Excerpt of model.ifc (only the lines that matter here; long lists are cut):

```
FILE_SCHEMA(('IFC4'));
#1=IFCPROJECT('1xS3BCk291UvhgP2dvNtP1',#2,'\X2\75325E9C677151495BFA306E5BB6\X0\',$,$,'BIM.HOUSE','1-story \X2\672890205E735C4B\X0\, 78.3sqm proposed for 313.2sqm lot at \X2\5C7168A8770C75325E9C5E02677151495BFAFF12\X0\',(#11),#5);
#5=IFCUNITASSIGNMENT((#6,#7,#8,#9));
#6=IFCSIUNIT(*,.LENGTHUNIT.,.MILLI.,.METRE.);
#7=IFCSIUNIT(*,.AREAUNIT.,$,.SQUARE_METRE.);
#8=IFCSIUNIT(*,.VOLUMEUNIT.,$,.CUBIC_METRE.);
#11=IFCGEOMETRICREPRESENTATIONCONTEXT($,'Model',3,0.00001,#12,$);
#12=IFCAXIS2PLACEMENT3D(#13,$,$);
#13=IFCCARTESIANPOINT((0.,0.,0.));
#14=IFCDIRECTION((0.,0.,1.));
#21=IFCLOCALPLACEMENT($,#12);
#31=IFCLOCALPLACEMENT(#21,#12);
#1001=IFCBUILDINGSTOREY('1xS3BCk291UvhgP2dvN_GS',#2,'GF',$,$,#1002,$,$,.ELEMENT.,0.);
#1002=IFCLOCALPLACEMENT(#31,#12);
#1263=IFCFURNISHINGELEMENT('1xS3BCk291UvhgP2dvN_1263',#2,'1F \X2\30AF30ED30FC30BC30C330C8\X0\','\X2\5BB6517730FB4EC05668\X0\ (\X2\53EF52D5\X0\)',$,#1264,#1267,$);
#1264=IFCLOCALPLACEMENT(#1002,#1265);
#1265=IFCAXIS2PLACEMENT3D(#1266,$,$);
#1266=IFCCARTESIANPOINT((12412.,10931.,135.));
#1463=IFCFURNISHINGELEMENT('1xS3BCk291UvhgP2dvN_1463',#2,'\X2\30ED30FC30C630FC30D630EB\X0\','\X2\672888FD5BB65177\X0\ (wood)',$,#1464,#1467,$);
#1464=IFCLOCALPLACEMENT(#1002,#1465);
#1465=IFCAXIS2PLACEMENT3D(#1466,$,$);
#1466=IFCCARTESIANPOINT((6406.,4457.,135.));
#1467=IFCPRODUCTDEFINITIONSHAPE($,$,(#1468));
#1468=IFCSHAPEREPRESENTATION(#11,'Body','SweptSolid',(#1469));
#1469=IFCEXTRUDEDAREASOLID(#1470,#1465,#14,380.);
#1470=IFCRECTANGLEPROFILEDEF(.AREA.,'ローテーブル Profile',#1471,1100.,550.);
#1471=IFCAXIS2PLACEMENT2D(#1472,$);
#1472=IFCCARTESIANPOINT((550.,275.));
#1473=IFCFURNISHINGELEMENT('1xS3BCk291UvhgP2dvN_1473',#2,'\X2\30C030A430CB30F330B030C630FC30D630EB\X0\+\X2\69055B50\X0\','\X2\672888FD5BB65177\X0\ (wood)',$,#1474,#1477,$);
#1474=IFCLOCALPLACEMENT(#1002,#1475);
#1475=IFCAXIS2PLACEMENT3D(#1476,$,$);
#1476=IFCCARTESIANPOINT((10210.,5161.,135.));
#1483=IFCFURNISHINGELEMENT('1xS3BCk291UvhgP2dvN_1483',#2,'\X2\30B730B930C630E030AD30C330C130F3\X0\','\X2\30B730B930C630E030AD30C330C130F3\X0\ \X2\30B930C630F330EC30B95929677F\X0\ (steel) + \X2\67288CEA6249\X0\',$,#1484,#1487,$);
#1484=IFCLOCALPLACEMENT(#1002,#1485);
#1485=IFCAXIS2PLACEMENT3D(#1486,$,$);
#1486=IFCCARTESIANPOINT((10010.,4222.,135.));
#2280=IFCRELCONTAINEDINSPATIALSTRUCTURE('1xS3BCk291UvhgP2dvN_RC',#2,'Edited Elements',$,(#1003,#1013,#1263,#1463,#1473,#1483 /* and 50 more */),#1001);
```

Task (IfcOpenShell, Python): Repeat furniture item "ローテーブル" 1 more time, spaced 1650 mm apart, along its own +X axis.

```python
import ifcopenshell
import ifcopenshell.api.geometry
import ifcopenshell.api.root
import ifcopenshell.util.element
import ifcopenshell.util.placement

model = ifcopenshell.open("model.ifc")


def reuse_history(source, copy):
    """copy_class also copies each property set's owner history, people and application; keep the originals."""
    for rel in copy.IsDefinedBy:
        if rel.is_a("IfcRelDefinesByProperties") and (history := rel.RelatingPropertyDefinition.OwnerHistory):
            rel.RelatingPropertyDefinition.OwnerHistory = source.OwnerHistory
            ifcopenshell.util.element.remove_deep2(model, history)


source = model.by_id(1463)
base = ifcopenshell.util.placement.get_local_placement(source.ObjectPlacement)
step = base[:3, 0] * 1650.0

for i in range(1, 2):
    copy = ifcopenshell.api.root.copy_class(model, product=source)
    copy.Representation = ifcopenshell.util.element.copy_deep(
        model, source.Representation, exclude=["IfcGeometricRepresentationContext", "IfcRepresentationMap"]
    )
    reuse_history(source, copy)
    matrix = base.copy()
    matrix[:3, 3] += i * step
    print("added at", matrix[:3, 3].round(3) + 0.0)
    ifcopenshell.api.geometry.edit_object_placement(model, product=copy, matrix=matrix, is_si=False)

model.write("model_rev.ifc")
```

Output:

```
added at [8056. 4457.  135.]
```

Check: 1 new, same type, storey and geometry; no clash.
